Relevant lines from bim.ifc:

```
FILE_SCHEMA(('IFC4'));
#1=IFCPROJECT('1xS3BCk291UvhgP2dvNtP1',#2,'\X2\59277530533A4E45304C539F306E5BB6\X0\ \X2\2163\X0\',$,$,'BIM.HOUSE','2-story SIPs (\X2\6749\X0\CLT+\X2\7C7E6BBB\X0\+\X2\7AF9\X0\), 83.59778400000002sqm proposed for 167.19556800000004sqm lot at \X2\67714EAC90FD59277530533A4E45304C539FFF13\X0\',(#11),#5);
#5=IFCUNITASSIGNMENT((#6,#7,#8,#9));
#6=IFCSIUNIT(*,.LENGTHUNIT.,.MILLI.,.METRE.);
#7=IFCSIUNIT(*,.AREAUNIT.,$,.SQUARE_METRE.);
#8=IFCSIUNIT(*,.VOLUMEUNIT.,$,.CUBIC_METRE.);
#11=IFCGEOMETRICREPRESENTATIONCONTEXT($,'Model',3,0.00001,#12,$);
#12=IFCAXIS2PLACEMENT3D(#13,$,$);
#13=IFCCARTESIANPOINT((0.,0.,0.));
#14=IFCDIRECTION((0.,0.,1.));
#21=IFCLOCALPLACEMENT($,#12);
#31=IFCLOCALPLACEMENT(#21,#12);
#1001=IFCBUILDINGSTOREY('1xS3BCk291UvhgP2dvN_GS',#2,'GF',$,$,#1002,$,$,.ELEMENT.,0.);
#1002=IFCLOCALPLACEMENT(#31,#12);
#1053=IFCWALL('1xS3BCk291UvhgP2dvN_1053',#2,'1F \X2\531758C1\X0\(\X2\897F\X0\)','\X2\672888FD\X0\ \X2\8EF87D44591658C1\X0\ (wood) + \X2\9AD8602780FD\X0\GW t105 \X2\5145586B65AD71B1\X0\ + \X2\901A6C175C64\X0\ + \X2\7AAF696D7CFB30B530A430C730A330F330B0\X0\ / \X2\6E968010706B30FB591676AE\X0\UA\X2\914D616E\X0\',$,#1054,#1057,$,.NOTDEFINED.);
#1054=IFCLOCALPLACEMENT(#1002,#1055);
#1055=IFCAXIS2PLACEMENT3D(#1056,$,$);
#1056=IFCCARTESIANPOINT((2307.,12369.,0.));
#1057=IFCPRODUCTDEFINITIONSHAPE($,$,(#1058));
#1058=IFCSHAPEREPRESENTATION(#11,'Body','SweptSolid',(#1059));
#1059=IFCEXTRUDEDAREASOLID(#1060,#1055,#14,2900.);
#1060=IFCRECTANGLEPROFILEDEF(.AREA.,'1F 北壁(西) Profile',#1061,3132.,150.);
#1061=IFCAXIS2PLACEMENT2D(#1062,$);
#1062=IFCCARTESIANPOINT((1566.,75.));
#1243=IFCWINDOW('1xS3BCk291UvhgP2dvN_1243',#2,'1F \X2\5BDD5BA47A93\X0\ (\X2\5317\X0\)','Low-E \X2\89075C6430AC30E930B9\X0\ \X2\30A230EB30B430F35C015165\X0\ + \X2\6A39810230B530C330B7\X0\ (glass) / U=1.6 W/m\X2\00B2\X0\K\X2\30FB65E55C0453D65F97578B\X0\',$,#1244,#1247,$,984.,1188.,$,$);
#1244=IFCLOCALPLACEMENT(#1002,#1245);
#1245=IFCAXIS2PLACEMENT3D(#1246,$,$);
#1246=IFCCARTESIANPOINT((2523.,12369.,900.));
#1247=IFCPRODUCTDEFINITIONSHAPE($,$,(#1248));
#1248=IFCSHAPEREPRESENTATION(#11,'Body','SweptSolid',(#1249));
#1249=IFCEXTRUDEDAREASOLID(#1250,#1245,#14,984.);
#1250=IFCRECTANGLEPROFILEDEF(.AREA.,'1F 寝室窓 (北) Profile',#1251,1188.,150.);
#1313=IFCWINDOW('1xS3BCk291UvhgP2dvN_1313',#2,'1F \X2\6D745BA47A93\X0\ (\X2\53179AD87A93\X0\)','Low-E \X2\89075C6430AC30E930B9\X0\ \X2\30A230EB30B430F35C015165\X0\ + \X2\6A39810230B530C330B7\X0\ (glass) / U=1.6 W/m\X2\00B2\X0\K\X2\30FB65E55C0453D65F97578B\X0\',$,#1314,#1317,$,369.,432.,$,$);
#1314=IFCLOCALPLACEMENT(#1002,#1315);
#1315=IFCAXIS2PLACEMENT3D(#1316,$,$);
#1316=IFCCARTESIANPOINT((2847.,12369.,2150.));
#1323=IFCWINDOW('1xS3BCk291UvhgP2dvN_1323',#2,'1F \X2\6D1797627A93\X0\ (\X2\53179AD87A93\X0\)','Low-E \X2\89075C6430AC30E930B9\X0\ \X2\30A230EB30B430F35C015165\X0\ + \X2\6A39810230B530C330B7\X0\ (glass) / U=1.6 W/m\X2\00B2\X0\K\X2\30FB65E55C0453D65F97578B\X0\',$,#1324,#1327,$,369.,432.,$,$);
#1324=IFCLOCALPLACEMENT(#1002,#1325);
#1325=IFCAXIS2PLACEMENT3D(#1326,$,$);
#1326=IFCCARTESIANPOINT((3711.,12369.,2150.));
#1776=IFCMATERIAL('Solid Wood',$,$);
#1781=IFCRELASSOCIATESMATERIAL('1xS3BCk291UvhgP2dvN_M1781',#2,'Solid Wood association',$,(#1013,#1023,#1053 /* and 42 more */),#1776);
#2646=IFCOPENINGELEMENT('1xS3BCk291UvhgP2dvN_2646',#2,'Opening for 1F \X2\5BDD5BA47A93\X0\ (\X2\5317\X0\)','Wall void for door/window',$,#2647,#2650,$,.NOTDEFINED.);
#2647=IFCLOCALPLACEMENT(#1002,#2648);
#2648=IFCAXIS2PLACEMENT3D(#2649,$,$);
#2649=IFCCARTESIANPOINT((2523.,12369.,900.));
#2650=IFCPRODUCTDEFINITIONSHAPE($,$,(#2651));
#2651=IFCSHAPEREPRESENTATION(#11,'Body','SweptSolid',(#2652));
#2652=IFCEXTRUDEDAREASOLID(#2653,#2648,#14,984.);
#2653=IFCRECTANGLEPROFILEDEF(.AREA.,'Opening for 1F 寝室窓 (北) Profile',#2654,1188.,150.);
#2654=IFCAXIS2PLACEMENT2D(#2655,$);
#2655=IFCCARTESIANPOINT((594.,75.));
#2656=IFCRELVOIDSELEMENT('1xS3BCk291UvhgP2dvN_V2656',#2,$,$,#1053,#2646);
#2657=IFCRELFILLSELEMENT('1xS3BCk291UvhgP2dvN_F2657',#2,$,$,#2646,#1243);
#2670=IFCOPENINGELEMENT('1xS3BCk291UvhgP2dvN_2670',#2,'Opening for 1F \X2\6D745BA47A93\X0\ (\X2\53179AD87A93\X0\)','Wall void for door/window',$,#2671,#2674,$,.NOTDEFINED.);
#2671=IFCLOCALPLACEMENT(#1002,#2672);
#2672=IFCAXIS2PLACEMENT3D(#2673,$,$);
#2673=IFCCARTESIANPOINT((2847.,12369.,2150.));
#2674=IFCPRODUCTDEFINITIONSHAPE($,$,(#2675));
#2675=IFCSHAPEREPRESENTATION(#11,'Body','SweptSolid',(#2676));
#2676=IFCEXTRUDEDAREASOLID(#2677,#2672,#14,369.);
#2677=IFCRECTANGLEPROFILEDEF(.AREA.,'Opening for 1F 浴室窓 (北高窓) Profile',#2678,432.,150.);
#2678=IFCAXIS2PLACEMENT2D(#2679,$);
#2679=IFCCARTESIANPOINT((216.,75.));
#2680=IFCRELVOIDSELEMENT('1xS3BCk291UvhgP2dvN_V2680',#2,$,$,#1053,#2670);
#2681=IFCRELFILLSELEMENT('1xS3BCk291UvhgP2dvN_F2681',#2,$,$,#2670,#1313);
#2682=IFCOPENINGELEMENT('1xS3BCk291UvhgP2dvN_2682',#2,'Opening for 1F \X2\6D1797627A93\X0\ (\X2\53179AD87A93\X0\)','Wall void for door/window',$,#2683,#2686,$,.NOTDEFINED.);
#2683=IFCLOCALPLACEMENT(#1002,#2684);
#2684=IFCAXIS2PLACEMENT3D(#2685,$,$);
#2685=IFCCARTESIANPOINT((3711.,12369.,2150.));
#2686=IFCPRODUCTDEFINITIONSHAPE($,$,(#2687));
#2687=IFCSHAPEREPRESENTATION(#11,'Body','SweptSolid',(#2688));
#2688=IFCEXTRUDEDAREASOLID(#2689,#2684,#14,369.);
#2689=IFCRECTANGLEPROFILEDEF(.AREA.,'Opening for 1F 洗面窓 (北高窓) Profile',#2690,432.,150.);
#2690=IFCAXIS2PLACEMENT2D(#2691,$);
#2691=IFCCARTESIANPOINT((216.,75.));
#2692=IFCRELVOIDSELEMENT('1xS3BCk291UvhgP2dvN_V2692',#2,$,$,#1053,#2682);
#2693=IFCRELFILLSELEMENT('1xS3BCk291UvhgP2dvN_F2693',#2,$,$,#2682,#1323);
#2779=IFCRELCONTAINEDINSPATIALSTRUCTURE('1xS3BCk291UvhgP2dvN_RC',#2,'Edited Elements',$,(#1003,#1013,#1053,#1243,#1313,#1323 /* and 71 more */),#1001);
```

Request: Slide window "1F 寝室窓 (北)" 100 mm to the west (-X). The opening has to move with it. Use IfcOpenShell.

```python
import ifcopenshell
import ifcopenshell.api.geometry
import ifcopenshell.util.placement

model = ifcopenshell.open("bim.ifc")

window = model.by_id(1243)
opening = window.FillsVoids[0].RelatingOpeningElement
wall = opening.VoidsElements[0].RelatingBuildingElement

wall_matrix = ifcopenshell.util.placement.get_local_placement(wall.ObjectPlacement)
shift = wall_matrix[:3, 0] * -100.0
before = ifcopenshell.util.placement.get_local_placement(window.ObjectPlacement)[:3, 3].copy()

# The window is not placed relative to its opening, so move both.
for product in (opening, window):
    matrix = ifcopenshell.util.placement.get_local_placement(product.ObjectPlacement)
    matrix[:3, 3] += shift
    ifcopenshell.api.geometry.edit_object_placement(model, product=product, matrix=matrix, is_si=False)

after = ifcopenshell.util.placement.get_local_placement(window.ObjectPlacement)[:3, 3]
print("window moved by", (after - before).round(3) + 0.0)

model.write("bim_updated.ifc")
```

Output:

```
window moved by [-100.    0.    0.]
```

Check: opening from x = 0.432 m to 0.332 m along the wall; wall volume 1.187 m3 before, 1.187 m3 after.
